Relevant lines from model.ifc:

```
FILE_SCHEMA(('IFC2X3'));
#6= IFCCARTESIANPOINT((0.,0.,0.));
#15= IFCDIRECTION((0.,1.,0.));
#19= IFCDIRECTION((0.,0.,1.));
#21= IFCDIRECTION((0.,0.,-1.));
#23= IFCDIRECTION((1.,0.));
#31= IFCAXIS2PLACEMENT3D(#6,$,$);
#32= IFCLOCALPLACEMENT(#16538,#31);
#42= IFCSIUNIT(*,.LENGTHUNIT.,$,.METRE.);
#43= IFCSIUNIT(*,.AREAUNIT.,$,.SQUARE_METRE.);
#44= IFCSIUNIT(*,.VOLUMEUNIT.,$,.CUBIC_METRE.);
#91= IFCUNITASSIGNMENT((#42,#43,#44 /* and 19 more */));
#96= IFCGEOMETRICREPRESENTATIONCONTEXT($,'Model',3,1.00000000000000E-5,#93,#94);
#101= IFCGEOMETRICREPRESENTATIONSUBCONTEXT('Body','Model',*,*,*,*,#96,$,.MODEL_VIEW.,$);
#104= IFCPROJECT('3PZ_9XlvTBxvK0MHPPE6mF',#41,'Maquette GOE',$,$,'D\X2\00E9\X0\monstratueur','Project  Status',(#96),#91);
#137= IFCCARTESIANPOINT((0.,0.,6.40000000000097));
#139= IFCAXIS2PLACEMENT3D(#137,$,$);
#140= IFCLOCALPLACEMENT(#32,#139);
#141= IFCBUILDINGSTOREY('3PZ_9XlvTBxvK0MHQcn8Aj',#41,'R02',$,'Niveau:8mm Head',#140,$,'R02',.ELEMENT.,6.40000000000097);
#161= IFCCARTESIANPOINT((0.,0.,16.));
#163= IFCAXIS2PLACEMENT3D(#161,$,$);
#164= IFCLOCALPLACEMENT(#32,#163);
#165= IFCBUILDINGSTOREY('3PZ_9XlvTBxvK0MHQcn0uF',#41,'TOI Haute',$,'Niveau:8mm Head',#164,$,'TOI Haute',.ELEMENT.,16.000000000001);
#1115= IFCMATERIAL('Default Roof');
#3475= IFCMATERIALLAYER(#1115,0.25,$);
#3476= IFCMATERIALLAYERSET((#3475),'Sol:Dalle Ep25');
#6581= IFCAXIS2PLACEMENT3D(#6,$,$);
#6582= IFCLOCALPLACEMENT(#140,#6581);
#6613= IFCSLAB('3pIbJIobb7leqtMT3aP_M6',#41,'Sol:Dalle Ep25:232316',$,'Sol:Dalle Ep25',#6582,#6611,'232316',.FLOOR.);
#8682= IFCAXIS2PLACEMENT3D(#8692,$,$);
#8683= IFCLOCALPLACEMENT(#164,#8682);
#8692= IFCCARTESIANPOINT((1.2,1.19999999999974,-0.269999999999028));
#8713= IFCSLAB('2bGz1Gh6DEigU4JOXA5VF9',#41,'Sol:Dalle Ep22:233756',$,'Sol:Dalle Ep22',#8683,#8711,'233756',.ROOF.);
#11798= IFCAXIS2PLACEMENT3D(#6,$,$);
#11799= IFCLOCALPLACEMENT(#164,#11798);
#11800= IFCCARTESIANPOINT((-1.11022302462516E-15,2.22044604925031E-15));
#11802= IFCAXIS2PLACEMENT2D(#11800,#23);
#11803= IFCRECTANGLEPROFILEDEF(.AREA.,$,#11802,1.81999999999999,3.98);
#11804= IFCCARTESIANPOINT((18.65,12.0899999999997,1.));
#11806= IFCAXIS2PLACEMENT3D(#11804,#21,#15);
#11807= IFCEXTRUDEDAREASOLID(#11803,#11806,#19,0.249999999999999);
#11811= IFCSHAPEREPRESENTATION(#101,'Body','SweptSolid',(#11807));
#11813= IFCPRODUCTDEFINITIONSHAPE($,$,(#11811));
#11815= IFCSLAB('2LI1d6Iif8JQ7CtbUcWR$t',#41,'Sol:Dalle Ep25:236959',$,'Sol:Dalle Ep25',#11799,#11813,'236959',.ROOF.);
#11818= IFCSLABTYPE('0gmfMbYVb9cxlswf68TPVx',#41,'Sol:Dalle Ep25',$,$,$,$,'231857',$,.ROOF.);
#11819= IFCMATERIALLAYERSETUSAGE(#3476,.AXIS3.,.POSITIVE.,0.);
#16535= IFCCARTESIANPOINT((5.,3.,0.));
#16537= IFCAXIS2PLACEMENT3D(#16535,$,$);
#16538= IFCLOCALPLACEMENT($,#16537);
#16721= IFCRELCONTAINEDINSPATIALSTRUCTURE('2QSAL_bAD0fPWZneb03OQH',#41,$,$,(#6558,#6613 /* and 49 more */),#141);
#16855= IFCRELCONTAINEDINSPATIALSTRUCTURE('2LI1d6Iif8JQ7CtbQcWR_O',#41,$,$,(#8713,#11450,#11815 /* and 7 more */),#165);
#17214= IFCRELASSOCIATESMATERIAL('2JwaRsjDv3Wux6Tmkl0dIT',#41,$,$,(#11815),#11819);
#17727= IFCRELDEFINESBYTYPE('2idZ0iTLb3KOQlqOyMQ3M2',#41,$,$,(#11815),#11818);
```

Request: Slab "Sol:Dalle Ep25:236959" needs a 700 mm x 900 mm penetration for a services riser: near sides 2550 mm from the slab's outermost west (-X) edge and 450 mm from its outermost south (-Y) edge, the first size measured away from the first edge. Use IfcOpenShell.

```python
import numpy as np
import ifcopenshell
import ifcopenshell.api.feature
import ifcopenshell.api.geometry
import ifcopenshell.api.root
import ifcopenshell.geom
import ifcopenshell.util.placement
import ifcopenshell.util.representation
import ifcopenshell.util.shape
import ifcopenshell.util.unit

model = ifcopenshell.open("model.ifc")
unit_scale = ifcopenshell.util.unit.calculate_unit_scale(model)
settings = ifcopenshell.geom.settings()


def volume(element):
    """Net volume in cubic metres, openings subtracted."""
    shape = ifcopenshell.geom.create_shape(settings, element)
    return ifcopenshell.util.shape.get_volume(shape.geometry)


slab = model.by_guid("2LI1d6Iif8JQ7CtbUcWR$t")
before = volume(slab)

# Extent in the slab's own axes, in metres. The edges named are its -X and -Y sides.
slab_shape = ifcopenshell.geom.create_shape(settings, slab)
vertices = ifcopenshell.util.shape.get_vertices(slab_shape.geometry)
x_min, y_min, bottom = vertices.min(axis=0)
top = vertices[:, 2].max()

opening = ifcopenshell.api.root.create_entity(model, ifc_class="IfcOpeningElement", name="Services riser opening")
context = ifcopenshell.util.representation.get_context(model, "Model", "Body", "MODEL_VIEW")
width, depth = 0.7, 0.9
outline = [(0.0, 0.0), (width, 0.0), (width, depth), (0.0, depth), (0.0, 0.0)]
# Overshoot both faces by 50 mm so the cut is clean.
shape = ifcopenshell.api.geometry.add_slab_representation(
    model, context=context, depth=top - bottom + 0.1, polyline=outline
)
ifcopenshell.api.geometry.assign_representation(model, product=opening, representation=shape)

matrix = ifcopenshell.util.placement.get_local_placement(slab.ObjectPlacement)
matrix[:, 3] = matrix @ np.append(np.array([x_min + 2.55, y_min + 0.45, bottom - 0.05]) / unit_scale, 1.0)
ifcopenshell.api.geometry.edit_object_placement(model, product=opening, matrix=matrix, is_si=False)
ifcopenshell.api.feature.add_feature(model, feature=opening, element=slab)

after = volume(slab)

print(f"slab volume {before:.3f} -> {after:.3f} m3")

model.write("model_v2.ifc")
```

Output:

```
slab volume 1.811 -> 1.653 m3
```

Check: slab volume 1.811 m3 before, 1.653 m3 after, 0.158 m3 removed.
